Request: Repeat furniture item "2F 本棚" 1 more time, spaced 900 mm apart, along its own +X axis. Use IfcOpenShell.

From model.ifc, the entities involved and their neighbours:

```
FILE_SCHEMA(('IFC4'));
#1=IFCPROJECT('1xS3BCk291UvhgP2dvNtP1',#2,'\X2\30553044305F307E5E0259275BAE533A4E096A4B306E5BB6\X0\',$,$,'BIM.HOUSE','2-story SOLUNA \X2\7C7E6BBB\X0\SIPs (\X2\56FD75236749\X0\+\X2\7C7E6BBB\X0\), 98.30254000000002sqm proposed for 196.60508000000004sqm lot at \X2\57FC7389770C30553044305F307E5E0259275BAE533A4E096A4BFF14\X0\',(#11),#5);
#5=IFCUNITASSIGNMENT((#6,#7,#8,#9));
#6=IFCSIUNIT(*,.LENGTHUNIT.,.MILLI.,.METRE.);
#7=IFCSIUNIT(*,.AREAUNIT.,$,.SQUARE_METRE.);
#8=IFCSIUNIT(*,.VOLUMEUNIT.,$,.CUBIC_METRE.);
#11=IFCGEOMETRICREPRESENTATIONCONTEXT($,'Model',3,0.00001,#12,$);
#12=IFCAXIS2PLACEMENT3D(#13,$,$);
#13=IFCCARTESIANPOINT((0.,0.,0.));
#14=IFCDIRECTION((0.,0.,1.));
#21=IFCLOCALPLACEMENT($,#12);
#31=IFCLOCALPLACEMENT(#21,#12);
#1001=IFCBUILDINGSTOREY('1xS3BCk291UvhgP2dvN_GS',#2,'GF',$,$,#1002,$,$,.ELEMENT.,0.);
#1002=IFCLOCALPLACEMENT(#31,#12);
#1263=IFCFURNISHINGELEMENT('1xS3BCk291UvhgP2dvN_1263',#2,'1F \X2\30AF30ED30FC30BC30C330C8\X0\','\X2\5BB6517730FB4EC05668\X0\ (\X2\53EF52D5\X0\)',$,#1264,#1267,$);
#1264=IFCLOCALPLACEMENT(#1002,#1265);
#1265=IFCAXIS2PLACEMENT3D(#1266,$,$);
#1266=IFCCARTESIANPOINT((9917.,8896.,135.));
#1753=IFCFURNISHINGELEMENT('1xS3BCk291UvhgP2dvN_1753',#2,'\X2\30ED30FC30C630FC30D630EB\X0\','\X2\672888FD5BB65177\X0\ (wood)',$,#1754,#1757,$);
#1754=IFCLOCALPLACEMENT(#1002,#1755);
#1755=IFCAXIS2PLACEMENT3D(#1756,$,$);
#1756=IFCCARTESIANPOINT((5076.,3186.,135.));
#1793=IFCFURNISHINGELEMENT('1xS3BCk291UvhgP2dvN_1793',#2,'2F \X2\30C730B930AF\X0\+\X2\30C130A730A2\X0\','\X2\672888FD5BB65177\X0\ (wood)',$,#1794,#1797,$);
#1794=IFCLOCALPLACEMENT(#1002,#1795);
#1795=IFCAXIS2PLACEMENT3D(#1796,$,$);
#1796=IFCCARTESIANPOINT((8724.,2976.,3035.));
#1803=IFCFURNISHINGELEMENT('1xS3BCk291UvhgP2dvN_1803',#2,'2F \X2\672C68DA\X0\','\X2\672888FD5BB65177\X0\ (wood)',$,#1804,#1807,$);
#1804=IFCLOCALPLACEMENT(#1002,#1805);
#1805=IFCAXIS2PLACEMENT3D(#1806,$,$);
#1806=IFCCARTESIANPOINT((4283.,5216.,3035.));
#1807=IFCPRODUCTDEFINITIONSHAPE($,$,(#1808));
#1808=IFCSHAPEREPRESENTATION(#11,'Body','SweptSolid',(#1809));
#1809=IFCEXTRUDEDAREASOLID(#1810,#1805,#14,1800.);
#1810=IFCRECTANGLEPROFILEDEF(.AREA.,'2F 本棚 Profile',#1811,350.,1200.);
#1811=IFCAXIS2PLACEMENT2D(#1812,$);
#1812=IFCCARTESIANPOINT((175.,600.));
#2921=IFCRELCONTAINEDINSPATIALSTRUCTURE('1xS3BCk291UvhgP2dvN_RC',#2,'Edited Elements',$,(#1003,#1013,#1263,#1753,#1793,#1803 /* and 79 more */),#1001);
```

```python
import ifcopenshell
import ifcopenshell.api.geometry
import ifcopenshell.api.root
import ifcopenshell.util.element
import ifcopenshell.util.placement

model = ifcopenshell.open("model.ifc")


def reuse_history(source, copy):
    """copy_class also copies each property set's owner history, people and application; keep the originals."""
    for rel in copy.IsDefinedBy:
        if rel.is_a("IfcRelDefinesByProperties") and (history := rel.RelatingPropertyDefinition.OwnerHistory):
            rel.RelatingPropertyDefinition.OwnerHistory = source.OwnerHistory
            ifcopenshell.util.element.remove_deep2(model, history)


source = model.by_id(1803)
base = ifcopenshell.util.placement.get_local_placement(source.ObjectPlacement)
step = base[:3, 0] * 900.0

for i in range(1, 2):
    copy = ifcopenshell.api.root.copy_class(model, product=source)
    copy.Representation = ifcopenshell.util.element.copy_deep(
        model, source.Representation, exclude=["IfcGeometricRepresentationContext", "IfcRepresentationMap"]
    )
    reuse_history(source, copy)
    matrix = base.copy()
    matrix[:3, 3] += i * step
    print("added at", matrix[:3, 3].round(3) + 0.0)
    ifcopenshell.api.geometry.edit_object_placement(model, product=copy, matrix=matrix, is_si=False)

model.write("model_rev.ifc")
```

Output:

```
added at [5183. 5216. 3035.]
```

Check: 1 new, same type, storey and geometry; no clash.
